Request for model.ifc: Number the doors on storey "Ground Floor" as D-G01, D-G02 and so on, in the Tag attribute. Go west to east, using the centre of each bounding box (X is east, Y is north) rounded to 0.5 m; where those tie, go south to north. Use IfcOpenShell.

First a look at what the model holds.

```python
import ifcopenshell
import ifcopenshell.util.element
import ifcopenshell.util.placement

model = ifcopenshell.open("model.ifc")
print(model.schema)
storey = next(s for s in model.by_type("IfcBuildingStorey") if s.Name == "Ground Floor")
doors = [e for e in ifcopenshell.util.element.get_decomposition(storey) if e.is_a("IfcDoor")]
for e in sorted(doors, key=lambda e: e.id()):
    origin = ifcopenshell.util.placement.get_local_placement(e.ObjectPlacement)[:3, 3]
    print(e.id(), e.Tag, e.Name, origin.round(2) + 0.0, sep=" | ")
```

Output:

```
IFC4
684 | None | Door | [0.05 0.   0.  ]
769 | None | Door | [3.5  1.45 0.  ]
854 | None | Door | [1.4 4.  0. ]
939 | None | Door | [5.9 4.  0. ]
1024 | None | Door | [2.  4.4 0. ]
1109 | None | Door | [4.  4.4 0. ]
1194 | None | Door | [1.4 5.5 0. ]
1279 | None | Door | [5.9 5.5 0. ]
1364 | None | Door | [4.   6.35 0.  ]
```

```python
import ifcopenshell
import ifcopenshell.geom
import ifcopenshell.util.element
import ifcopenshell.util.shape

model = ifcopenshell.open("model.ifc")
settings = ifcopenshell.geom.settings()
settings.set("use-world-coords", True)


def centre(element):
    shape = ifcopenshell.geom.create_shape(settings, element)
    return ifcopenshell.util.shape.get_bbox_centroid(shape.geometry)


storey = next(s for s in model.by_type("IfcBuildingStorey") if s.Name == "Ground Floor")
doors = [e for e in ifcopenshell.util.element.get_decomposition(storey) if e.is_a("IfcDoor")]

# Insertion points can sit at a corner or the storey origin, so sort by the geometry (in metres).
centres = {e: centre(e) for e in doors}
doors.sort(key=lambda e: (round(centres[e][0] / 0.5), centres[e][1]))

for i, e in enumerate(doors, start=1):
    number = f"D-G{i:02d}"
    e.Tag = number
    print(e.id(), number)

model.write("model_rev.ifc")
```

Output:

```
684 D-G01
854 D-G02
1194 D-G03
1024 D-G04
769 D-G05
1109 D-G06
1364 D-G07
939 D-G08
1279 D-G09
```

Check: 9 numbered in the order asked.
